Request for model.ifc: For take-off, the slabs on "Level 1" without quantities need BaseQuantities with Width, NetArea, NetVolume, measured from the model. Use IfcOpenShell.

First a look at what the model holds.

```python
import ifcopenshell
import ifcopenshell.util.element
import ifcopenshell.util.unit

model = ifcopenshell.open("model.ifc")
print(model.schema)
for unit_type in ("LENGTHUNIT", "AREAUNIT", "VOLUMEUNIT"):
    print(unit_type, ifcopenshell.util.unit.calculate_unit_scale(model, unit_type))
storey = next(s for s in model.by_type("IfcBuildingStorey") if s.Name == "Level 1")
slabs = [e for e in ifcopenshell.util.element.get_decomposition(storey) if e.is_a("IfcSlab")]
for e in sorted(slabs, key=lambda e: e.id()):
    print(e.id(), e.is_a(), e.Name, list(ifcopenshell.util.element.get_psets(e, qtos_only=True)), sep=" | ")
```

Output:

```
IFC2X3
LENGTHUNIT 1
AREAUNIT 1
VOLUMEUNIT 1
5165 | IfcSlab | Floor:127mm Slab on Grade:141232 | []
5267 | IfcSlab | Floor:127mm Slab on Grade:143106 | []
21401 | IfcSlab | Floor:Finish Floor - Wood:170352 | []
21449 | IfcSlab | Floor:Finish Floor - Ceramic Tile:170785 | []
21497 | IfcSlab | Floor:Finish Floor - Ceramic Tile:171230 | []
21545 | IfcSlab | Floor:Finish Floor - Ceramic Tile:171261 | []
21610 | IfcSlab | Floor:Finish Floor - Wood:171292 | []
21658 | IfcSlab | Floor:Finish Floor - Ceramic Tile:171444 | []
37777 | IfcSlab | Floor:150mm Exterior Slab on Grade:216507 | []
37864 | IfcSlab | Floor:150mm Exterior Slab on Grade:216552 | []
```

```python
import ifcopenshell
import ifcopenshell.api.pset
import ifcopenshell.geom
import ifcopenshell.util.element
import ifcopenshell.util.shape
import ifcopenshell.util.unit

model = ifcopenshell.open("model.ifc")
unit_scale = ifcopenshell.util.unit.calculate_unit_scale(model)
area_scale = ifcopenshell.util.unit.calculate_unit_scale(model, "AREAUNIT")
volume_scale = ifcopenshell.util.unit.calculate_unit_scale(model, "VOLUMEUNIT")
settings = ifcopenshell.geom.settings()

storey = next(s for s in model.by_type("IfcBuildingStorey") if s.Name == "Level 1")
slabs = [e for e in ifcopenshell.util.element.get_decomposition(storey) if e.is_a("IfcSlab")]

for e in sorted(slabs, key=lambda e: e.id()):
    if ifcopenshell.util.element.get_psets(e, qtos_only=True, should_inherit=False):
        continue
    # Geometry comes back in metres, in the element's own axes.
    shape = ifcopenshell.geom.create_shape(settings, e)
    values = {
        "Width": ifcopenshell.util.shape.get_z(shape.geometry) / unit_scale,
        "NetArea": ifcopenshell.util.shape.get_footprint_area(shape.geometry) / area_scale,
        "NetVolume": ifcopenshell.util.shape.get_volume(shape.geometry) / volume_scale,
    }
    qto = ifcopenshell.api.pset.add_qto(model, product=e, name="BaseQuantities")
    ifcopenshell.api.pset.edit_qto(model, qto=qto, properties=values)
    print(e.id(), {k: round(v, 3) for k, v in values.items()})

model.write("model-out.ifc")
```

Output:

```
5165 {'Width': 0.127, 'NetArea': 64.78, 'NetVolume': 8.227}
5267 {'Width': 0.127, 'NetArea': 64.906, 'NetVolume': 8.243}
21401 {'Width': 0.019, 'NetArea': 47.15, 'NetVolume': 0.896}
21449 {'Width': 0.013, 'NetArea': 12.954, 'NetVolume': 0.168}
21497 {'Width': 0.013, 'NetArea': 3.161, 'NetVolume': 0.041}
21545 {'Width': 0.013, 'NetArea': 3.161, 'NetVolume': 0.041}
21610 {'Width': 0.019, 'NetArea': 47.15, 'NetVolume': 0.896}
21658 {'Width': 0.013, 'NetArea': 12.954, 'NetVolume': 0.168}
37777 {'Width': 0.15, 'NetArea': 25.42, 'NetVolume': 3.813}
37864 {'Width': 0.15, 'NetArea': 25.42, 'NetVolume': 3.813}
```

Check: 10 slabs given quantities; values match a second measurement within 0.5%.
